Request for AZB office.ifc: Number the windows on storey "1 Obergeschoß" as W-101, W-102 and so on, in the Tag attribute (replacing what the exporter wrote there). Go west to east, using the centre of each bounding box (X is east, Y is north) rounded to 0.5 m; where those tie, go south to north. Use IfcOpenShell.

First a look at what the model holds.

```python
import ifcopenshell
import ifcopenshell.util.element
import ifcopenshell.util.placement

model = ifcopenshell.open("AZB office.ifc")
print(model.schema)
storey = next(s for s in model.by_type("IfcBuildingStorey") if s.Name == "1 Obergeschoß")
windows = [e for e in ifcopenshell.util.element.get_decomposition(storey) if e.is_a("IfcWindow")]
for e in sorted(windows, key=lambda e: e.id()):
    origin = ifcopenshell.util.placement.get_local_placement(e.ObjectPlacement)[:3, 3]
    print(e.id(), e.Tag, e.Name, origin.round(2) + 0.0, sep=" | ")
```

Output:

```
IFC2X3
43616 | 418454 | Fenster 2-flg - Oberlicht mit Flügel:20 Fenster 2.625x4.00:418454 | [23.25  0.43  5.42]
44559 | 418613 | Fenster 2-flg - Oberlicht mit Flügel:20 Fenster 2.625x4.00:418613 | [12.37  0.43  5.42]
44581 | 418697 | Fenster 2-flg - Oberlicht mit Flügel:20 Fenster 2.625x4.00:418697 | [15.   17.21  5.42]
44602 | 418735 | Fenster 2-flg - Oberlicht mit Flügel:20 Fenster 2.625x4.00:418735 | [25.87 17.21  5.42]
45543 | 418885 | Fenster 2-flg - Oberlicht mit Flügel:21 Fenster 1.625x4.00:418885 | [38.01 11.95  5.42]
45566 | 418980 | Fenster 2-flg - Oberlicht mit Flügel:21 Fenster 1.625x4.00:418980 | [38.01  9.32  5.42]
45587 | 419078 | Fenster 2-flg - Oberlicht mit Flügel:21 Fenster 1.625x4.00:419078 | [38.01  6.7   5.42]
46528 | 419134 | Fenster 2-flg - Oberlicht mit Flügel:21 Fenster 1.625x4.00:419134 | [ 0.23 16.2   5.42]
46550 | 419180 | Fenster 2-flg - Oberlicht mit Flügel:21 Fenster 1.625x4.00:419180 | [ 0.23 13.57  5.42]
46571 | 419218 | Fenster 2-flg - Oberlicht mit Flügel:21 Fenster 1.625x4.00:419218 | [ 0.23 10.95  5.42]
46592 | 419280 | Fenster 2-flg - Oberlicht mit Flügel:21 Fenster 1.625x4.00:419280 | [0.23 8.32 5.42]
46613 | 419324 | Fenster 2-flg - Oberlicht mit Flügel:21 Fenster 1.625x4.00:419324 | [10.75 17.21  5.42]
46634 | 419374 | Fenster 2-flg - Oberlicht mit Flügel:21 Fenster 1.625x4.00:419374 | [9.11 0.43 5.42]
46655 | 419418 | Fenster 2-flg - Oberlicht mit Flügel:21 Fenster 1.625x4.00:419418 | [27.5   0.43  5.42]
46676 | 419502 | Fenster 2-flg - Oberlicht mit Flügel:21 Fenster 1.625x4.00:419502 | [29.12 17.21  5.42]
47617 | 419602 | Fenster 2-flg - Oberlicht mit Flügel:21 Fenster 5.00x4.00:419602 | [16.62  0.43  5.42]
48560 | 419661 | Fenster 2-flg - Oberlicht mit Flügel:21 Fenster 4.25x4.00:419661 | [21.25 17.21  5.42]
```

```python
import ifcopenshell
import ifcopenshell.geom
import ifcopenshell.util.element
import ifcopenshell.util.shape

model = ifcopenshell.open("AZB office.ifc")
settings = ifcopenshell.geom.settings()
settings.set("use-world-coords", True)


def centre(element):
    shape = ifcopenshell.geom.create_shape(settings, element)
    return ifcopenshell.util.shape.get_bbox_centroid(shape.geometry)


storey = next(s for s in model.by_type("IfcBuildingStorey") if s.Name == "1 Obergeschoß")
windows = [e for e in ifcopenshell.util.element.get_decomposition(storey) if e.is_a("IfcWindow")]

# Insertion points can sit at a corner or the storey origin, so sort by the geometry (in metres).
centres = {e: centre(e) for e in windows}
windows.sort(key=lambda e: (round(centres[e][0] / 0.5), centres[e][1]))

for i, e in enumerate(windows, start=1):
    number = f"W-1{i:02d}"
    e.Tag = number
    print(e.id(), number)

model.write("AZB office-out.ifc")
```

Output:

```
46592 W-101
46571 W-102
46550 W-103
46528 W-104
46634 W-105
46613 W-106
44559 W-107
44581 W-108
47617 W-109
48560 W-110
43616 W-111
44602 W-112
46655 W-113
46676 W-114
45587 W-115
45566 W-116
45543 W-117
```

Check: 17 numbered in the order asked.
